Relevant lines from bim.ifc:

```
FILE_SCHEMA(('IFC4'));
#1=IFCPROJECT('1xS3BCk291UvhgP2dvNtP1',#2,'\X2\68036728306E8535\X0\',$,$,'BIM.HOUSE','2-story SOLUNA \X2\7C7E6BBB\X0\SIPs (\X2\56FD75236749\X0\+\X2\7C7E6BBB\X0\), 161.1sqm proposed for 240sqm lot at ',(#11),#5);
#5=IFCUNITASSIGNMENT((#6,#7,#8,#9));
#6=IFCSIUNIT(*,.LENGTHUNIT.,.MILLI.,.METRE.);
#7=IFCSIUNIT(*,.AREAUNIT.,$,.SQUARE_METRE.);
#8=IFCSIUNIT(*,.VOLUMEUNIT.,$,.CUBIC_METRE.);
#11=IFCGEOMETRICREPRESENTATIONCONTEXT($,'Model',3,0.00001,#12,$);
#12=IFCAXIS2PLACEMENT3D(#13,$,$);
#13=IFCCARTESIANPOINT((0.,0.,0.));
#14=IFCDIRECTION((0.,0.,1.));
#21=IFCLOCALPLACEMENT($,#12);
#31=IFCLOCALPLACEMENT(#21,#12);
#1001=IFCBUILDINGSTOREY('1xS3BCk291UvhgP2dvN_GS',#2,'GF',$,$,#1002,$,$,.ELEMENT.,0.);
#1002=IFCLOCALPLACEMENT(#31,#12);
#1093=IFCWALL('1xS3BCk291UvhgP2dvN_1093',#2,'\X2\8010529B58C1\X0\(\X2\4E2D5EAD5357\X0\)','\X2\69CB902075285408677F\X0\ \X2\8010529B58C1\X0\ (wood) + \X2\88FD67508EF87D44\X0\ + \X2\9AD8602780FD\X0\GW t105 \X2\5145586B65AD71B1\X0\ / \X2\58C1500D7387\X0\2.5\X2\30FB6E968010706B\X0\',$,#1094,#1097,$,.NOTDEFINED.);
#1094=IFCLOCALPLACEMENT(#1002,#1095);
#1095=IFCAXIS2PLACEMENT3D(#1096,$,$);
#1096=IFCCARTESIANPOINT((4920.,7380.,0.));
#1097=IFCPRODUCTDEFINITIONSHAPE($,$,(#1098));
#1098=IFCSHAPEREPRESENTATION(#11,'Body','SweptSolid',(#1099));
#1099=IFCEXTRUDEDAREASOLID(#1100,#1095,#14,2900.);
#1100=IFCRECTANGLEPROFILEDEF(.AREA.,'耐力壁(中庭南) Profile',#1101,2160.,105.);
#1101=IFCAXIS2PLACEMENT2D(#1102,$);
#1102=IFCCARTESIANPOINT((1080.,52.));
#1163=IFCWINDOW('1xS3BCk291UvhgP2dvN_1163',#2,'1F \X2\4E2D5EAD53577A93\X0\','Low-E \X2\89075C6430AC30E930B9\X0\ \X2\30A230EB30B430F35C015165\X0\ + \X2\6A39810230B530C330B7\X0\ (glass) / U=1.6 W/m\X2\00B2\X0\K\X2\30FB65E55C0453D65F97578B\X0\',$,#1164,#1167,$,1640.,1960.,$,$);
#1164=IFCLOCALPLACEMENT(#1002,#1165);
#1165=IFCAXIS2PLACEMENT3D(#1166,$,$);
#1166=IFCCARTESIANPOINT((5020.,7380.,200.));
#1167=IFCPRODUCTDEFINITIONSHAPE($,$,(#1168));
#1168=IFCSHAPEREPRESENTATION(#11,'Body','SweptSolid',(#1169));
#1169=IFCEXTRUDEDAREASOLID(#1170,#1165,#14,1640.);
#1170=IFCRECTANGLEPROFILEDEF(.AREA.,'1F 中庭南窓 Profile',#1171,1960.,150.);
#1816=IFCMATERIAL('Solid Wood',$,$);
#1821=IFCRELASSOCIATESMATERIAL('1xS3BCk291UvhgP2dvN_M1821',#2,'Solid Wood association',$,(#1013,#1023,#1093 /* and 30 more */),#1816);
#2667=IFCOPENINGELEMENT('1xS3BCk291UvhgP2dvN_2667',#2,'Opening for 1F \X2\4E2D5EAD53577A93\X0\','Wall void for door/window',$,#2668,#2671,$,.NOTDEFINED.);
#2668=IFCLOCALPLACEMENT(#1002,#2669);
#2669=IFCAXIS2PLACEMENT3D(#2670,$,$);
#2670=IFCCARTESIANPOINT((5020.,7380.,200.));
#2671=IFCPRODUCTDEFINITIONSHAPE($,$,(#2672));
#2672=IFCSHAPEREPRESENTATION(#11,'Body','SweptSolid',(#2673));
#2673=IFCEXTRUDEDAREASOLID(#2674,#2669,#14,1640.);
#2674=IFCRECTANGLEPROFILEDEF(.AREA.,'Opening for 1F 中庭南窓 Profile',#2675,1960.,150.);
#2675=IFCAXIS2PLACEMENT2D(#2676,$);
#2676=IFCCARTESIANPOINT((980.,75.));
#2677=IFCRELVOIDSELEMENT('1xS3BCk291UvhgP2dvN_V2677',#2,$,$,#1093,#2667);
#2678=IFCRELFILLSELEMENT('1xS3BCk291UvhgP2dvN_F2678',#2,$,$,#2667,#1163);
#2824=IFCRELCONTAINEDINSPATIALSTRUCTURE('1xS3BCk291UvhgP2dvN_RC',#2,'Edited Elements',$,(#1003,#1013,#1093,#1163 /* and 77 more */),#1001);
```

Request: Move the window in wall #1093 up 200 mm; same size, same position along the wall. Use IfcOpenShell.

```python
import numpy as np
import ifcopenshell
import ifcopenshell.api.geometry
import ifcopenshell.util.placement
import ifcopenshell.util.unit

model = ifcopenshell.open("bim.ifc")
unit_scale = ifcopenshell.util.unit.calculate_unit_scale(model)

window = model.by_guid("1xS3BCk291UvhgP2dvN_1163")
opening = window.FillsVoids[0].RelatingOpeningElement
dz = 200.0

shift = np.array([0.0, 0.0, dz])
# The window is not placed relative to its opening, so move both.
for product in (opening, window):
    matrix = ifcopenshell.util.placement.get_local_placement(product.ObjectPlacement)
    matrix[:3, 3] += shift
    ifcopenshell.api.geometry.edit_object_placement(model, product=product, matrix=matrix, is_si=False)

print(f"moved by {dz * unit_scale:+.3f} m")

model.write("bim_v2.ifc")
```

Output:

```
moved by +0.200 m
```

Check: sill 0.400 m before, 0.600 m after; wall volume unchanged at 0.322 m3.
